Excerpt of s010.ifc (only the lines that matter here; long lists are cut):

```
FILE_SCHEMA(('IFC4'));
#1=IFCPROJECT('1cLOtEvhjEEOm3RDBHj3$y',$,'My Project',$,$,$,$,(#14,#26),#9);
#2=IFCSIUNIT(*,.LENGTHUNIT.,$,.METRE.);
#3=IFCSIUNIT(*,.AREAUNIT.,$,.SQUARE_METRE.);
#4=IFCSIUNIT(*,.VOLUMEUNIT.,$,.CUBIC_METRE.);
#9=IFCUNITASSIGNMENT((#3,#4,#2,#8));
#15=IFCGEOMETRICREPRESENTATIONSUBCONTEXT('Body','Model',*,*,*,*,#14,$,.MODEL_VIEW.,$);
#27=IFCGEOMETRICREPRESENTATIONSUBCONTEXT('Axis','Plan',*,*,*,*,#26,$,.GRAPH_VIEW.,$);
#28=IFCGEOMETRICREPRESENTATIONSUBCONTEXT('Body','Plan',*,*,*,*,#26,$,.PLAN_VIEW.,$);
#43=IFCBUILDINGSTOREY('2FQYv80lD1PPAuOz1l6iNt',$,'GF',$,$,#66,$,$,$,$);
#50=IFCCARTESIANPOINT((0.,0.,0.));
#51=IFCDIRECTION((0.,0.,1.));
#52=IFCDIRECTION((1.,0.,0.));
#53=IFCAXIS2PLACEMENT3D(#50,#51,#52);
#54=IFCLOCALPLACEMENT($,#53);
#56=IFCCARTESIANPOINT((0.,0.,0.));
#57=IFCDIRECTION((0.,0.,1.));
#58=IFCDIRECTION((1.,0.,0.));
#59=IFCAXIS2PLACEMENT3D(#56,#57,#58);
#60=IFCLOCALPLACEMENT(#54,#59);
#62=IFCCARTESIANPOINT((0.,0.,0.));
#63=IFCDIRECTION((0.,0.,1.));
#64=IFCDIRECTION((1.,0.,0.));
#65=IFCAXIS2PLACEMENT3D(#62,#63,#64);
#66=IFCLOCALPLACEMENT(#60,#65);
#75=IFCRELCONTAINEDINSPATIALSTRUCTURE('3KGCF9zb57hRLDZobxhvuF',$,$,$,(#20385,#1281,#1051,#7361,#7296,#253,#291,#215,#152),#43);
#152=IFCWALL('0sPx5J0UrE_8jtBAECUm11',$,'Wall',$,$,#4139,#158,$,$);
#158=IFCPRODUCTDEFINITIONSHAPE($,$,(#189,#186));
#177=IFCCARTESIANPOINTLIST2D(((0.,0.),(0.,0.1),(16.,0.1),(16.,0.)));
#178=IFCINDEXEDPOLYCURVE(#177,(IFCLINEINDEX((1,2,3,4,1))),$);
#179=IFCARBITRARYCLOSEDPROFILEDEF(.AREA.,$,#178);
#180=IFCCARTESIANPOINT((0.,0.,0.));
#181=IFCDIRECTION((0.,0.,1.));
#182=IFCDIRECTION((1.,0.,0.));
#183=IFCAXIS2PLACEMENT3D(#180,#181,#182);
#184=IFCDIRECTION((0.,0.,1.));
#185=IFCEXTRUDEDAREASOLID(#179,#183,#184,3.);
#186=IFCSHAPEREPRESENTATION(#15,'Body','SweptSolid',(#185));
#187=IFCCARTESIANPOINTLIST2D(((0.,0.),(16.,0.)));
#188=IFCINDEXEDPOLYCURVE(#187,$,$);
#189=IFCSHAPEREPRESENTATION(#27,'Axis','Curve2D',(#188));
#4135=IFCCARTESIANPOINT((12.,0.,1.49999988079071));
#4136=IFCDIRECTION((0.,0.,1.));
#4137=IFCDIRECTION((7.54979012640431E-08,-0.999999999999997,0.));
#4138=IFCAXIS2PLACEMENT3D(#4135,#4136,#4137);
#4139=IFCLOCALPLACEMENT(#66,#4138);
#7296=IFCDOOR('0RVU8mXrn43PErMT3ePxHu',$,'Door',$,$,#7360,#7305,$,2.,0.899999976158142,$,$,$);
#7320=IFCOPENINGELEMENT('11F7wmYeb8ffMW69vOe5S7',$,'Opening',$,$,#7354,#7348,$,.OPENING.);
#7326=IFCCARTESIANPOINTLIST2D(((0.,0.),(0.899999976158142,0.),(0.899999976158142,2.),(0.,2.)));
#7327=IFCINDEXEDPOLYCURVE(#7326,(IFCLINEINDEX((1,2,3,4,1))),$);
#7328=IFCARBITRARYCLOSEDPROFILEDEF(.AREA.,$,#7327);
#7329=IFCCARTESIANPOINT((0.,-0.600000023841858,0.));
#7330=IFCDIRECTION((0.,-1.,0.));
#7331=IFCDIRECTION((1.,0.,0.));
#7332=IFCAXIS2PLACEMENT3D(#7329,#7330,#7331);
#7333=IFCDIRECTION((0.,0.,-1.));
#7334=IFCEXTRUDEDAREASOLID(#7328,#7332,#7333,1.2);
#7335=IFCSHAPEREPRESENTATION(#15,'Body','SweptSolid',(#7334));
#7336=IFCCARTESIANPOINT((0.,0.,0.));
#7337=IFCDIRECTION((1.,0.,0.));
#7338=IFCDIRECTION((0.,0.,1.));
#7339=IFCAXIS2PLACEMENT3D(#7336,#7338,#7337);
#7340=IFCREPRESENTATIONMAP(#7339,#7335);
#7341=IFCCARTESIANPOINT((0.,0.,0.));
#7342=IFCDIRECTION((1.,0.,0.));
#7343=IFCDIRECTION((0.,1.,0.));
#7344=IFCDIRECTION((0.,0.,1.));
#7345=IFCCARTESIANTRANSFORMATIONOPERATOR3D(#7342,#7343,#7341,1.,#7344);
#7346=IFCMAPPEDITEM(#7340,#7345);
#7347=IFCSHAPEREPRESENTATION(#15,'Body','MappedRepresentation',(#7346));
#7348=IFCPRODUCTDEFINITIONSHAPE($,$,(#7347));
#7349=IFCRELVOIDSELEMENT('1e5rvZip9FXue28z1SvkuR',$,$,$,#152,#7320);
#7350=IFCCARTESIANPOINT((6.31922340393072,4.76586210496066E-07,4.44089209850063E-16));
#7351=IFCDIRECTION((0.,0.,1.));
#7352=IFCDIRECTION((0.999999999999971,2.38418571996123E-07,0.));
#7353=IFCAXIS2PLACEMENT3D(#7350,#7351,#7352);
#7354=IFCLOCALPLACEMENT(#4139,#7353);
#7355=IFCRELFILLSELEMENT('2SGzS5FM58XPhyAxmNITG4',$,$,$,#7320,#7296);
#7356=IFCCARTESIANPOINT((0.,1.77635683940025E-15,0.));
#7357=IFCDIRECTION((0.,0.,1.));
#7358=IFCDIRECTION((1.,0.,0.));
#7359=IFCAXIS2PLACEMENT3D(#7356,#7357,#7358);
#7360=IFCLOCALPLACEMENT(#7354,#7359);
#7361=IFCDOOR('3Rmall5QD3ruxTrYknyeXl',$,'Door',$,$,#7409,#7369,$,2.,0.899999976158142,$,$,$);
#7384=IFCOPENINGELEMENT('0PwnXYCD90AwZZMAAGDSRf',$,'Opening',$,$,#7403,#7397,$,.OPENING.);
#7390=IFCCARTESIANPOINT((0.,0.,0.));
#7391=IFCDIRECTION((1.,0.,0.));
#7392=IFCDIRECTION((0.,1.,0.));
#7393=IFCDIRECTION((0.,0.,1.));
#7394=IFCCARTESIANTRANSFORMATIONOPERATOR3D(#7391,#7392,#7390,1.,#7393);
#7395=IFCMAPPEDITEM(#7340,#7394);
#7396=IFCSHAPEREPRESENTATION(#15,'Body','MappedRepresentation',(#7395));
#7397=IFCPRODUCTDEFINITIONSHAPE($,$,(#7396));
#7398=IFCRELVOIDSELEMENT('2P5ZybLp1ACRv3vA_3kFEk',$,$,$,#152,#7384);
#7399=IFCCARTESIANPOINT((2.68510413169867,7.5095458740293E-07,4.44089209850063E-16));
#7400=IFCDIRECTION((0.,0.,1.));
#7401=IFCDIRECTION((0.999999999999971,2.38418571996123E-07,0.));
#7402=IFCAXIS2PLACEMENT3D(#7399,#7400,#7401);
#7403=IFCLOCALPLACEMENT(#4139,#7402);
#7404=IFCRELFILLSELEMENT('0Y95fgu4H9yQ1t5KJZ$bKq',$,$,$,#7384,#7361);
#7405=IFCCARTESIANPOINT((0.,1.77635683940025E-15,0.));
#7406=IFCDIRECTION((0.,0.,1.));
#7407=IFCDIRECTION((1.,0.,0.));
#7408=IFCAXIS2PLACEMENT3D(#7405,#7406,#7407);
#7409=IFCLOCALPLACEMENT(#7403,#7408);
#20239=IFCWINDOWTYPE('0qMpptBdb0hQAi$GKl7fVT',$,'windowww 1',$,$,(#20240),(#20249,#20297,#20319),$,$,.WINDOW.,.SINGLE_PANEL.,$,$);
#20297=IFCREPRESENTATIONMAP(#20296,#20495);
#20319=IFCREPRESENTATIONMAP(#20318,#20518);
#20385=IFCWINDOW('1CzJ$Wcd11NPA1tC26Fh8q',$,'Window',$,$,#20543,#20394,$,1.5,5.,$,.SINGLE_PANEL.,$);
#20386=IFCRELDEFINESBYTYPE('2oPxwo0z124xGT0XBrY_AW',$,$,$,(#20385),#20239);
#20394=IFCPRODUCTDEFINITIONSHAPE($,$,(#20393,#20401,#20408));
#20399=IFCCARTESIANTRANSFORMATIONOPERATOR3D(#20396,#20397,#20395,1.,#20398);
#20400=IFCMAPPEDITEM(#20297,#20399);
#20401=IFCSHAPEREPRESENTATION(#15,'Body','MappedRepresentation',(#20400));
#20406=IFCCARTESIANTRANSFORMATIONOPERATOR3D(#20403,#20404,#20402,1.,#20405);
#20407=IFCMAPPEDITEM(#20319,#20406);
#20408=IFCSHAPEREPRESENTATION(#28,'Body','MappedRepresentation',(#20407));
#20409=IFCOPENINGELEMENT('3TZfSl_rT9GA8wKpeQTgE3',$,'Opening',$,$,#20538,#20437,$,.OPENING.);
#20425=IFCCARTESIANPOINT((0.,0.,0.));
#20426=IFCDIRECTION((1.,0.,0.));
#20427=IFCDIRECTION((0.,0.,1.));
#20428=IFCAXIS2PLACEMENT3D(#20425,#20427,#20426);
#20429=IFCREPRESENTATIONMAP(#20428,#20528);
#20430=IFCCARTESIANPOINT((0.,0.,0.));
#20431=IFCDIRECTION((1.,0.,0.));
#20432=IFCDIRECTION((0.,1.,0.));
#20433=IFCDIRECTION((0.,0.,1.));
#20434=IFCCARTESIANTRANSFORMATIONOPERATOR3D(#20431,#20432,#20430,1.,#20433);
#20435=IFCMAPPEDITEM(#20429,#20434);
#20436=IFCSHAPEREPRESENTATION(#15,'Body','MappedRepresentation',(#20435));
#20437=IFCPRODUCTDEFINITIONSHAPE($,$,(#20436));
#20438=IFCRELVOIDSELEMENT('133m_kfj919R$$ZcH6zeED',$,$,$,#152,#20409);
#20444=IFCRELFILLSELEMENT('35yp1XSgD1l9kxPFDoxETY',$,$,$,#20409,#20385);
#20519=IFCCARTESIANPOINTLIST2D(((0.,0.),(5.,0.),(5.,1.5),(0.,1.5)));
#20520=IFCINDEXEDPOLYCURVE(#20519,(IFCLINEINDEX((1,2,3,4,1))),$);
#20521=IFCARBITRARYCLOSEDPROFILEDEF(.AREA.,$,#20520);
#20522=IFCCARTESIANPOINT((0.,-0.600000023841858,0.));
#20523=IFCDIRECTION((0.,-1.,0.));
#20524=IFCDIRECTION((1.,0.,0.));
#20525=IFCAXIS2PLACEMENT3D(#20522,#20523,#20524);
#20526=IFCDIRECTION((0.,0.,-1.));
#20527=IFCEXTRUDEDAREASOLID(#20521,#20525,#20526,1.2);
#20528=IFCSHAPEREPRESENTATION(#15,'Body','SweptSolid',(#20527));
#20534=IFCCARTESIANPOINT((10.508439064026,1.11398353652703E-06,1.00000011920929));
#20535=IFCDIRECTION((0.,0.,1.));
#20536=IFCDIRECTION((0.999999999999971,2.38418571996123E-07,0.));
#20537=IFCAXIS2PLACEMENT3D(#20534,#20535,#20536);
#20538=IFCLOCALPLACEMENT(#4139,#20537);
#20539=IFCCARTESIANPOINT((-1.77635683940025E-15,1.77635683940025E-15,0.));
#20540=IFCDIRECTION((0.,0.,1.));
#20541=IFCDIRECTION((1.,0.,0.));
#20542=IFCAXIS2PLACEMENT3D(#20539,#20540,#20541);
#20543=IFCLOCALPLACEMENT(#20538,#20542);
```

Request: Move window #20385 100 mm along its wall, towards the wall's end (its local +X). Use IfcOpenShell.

```python
import ifcopenshell
import ifcopenshell.api.geometry
import ifcopenshell.util.placement

model = ifcopenshell.open("s010.ifc")

window = model.by_guid("1CzJ$Wcd11NPA1tC26Fh8q")
opening = window.FillsVoids[0].RelatingOpeningElement
wall = opening.VoidsElements[0].RelatingBuildingElement

wall_matrix = ifcopenshell.util.placement.get_local_placement(wall.ObjectPlacement)
shift = wall_matrix[:3, 0] * 0.1
before = ifcopenshell.util.placement.get_local_placement(window.ObjectPlacement)[:3, 3].copy()

# The window is placed relative to its opening, so it follows when the opening moves.
matrix = ifcopenshell.util.placement.get_local_placement(opening.ObjectPlacement)
matrix[:3, 3] += shift
ifcopenshell.api.geometry.edit_object_placement(
    model, product=opening, matrix=matrix, is_si=False, should_transform_children=True
)

after = ifcopenshell.util.placement.get_local_placement(window.ObjectPlacement)[:3, 3]
print("window moved by", (after - before).round(3) + 0.0)

model.write("s010_rev.ifc")
```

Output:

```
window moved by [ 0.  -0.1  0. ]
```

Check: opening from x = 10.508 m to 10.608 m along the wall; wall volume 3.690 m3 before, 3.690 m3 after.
